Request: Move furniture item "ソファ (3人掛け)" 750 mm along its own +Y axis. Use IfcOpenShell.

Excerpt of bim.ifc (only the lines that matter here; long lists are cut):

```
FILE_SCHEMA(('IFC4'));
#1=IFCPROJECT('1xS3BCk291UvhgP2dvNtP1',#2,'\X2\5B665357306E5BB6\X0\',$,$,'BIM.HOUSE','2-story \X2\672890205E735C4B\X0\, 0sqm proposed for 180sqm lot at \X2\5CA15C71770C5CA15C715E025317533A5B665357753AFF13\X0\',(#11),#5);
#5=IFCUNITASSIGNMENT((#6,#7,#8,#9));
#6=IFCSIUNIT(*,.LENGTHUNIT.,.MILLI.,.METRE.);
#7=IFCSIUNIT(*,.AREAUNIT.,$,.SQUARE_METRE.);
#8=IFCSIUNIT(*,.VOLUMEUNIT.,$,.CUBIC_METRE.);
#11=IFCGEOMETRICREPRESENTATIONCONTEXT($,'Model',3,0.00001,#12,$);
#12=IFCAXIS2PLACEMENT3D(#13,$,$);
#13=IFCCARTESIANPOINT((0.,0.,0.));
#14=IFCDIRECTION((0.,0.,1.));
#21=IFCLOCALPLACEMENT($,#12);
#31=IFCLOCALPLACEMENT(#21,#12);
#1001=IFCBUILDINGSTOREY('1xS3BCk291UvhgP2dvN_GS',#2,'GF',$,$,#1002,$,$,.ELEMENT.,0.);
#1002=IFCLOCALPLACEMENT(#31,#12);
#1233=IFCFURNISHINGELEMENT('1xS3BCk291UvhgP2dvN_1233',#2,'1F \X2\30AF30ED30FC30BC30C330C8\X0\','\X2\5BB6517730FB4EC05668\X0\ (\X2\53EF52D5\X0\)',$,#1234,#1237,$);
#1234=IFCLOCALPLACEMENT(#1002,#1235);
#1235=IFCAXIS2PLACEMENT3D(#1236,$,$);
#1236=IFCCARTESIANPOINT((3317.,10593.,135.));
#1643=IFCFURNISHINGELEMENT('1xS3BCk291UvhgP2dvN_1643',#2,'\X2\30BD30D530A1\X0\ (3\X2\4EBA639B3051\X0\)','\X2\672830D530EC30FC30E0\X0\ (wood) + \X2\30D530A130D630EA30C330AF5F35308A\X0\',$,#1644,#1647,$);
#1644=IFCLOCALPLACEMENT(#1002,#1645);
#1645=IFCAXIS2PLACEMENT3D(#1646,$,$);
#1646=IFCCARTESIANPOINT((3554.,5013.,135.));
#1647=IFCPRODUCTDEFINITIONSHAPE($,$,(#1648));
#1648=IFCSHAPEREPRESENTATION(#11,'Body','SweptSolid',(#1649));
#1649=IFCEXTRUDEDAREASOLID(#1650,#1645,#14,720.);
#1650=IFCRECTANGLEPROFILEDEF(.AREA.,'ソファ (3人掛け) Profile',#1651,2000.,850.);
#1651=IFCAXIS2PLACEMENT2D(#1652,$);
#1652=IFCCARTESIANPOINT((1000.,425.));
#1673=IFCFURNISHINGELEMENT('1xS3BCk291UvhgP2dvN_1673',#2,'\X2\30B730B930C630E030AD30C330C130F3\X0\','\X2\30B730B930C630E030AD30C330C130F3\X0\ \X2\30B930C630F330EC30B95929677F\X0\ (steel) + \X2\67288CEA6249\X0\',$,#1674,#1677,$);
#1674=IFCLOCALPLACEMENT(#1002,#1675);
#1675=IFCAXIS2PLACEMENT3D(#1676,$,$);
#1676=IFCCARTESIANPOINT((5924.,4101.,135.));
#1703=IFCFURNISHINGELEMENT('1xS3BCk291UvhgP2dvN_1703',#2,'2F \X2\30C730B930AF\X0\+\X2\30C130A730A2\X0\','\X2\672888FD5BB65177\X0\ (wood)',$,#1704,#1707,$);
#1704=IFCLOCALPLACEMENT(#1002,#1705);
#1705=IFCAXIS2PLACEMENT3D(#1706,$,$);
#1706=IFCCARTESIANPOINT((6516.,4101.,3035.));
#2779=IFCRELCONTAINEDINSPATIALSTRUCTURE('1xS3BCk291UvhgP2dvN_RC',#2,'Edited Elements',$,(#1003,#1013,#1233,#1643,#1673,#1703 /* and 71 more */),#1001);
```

```python
import ifcopenshell
import ifcopenshell.api.geometry
import ifcopenshell.util.placement

model = ifcopenshell.open("bim.ifc")

item = model.by_guid("1xS3BCk291UvhgP2dvN_1643")
matrix = ifcopenshell.util.placement.get_local_placement(item.ObjectPlacement)
matrix[:3, 3] += matrix[:3, 1] * 750.0
ifcopenshell.api.geometry.edit_object_placement(model, product=item, matrix=matrix, is_si=False)

print(ifcopenshell.util.placement.get_local_placement(item.ObjectPlacement).round(3) + 0.0)

model.write("bim_rev.ifc")
```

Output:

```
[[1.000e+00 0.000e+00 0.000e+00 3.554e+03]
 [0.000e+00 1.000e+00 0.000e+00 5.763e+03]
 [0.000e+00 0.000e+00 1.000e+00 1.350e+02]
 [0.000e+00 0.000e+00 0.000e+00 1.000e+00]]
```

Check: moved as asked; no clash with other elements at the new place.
